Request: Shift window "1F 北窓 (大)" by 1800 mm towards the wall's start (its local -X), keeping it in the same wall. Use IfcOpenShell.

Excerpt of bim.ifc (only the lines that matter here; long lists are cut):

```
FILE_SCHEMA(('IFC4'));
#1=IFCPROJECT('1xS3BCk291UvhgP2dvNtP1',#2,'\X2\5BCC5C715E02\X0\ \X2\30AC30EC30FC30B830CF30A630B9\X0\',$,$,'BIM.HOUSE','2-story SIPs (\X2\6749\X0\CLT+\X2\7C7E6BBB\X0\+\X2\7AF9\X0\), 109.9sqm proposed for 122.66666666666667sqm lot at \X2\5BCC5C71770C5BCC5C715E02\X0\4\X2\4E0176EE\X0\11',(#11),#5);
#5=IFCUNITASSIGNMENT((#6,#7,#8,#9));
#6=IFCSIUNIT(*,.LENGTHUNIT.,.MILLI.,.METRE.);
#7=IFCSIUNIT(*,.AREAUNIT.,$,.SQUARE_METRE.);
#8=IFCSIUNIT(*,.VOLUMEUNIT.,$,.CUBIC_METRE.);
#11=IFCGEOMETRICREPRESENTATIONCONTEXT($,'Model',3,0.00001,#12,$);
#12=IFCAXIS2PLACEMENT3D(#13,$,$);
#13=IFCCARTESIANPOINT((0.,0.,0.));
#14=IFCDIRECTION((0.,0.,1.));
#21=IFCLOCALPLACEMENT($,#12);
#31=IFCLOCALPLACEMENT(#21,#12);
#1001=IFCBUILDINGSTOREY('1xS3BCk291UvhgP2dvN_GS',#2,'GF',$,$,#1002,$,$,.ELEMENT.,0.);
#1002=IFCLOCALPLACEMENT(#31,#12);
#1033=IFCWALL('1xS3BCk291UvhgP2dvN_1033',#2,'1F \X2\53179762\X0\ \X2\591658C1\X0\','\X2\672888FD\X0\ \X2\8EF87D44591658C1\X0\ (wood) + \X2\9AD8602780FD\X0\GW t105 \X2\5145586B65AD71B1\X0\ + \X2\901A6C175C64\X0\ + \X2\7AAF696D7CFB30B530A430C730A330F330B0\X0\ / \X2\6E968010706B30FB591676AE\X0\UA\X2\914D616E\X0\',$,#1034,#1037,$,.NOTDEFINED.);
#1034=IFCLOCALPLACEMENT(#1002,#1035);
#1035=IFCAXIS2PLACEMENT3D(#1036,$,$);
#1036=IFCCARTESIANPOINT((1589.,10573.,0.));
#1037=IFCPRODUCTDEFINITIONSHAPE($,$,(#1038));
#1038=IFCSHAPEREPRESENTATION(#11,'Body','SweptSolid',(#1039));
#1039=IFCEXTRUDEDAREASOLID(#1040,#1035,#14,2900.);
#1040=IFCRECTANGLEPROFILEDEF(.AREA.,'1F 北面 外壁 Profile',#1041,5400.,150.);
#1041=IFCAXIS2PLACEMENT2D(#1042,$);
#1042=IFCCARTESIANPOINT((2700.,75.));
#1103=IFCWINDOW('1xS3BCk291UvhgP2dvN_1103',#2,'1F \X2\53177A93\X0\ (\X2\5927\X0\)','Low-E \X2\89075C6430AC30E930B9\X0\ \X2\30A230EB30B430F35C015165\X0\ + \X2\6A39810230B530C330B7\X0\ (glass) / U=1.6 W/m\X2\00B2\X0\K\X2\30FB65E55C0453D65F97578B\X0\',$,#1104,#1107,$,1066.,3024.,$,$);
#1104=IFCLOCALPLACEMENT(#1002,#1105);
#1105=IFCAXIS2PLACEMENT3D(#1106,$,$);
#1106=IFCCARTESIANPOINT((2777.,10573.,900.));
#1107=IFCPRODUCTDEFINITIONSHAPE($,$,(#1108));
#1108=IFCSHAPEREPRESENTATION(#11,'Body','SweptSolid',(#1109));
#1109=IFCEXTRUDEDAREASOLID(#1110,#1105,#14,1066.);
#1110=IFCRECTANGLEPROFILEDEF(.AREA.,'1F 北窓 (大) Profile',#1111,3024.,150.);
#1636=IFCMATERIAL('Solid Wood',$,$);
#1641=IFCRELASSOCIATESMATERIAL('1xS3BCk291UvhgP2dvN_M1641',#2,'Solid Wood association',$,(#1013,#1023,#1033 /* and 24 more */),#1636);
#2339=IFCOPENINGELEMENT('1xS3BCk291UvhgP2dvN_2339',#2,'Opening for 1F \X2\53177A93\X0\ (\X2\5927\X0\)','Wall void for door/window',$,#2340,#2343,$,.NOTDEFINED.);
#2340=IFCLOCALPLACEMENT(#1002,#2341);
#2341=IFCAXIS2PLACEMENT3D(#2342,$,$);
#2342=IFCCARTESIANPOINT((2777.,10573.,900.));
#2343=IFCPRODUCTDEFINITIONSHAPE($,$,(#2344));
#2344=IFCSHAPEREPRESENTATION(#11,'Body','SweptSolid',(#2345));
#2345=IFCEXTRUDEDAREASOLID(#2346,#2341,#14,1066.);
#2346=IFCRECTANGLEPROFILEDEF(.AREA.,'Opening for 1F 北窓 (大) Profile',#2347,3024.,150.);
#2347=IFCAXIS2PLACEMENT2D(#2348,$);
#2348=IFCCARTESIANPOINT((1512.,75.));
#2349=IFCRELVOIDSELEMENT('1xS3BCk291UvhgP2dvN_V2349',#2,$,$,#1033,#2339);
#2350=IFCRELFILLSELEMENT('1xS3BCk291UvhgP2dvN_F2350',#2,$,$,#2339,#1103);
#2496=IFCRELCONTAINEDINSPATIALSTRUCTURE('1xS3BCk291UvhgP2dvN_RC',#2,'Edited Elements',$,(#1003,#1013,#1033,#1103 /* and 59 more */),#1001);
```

```python
import ifcopenshell
import ifcopenshell.api.geometry
import ifcopenshell.util.placement
import ifcopenshell.util.unit

model = ifcopenshell.open("bim.ifc")
unit_scale = ifcopenshell.util.unit.calculate_unit_scale(model)

window = model.by_guid("1xS3BCk291UvhgP2dvN_1103")
opening = window.FillsVoids[0].RelatingOpeningElement
wall = opening.VoidsElements[0].RelatingBuildingElement

wall_matrix = ifcopenshell.util.placement.get_local_placement(wall.ObjectPlacement)
shift = wall_matrix[:3, 0] * -1.8 / unit_scale
before = ifcopenshell.util.placement.get_local_placement(window.ObjectPlacement)[:3, 3].copy()

# The window is not placed relative to its opening, so move both.
for product in (opening, window):
    matrix = ifcopenshell.util.placement.get_local_placement(product.ObjectPlacement)
    matrix[:3, 3] += shift
    ifcopenshell.api.geometry.edit_object_placement(model, product=product, matrix=matrix, is_si=False)

after = ifcopenshell.util.placement.get_local_placement(window.ObjectPlacement)[:3, 3]
print("window moved by", (after - before).round(3) + 0.0)

model.write("bim_edited.ifc")
```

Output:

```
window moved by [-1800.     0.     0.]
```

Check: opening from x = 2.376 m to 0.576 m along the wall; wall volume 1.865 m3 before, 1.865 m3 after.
